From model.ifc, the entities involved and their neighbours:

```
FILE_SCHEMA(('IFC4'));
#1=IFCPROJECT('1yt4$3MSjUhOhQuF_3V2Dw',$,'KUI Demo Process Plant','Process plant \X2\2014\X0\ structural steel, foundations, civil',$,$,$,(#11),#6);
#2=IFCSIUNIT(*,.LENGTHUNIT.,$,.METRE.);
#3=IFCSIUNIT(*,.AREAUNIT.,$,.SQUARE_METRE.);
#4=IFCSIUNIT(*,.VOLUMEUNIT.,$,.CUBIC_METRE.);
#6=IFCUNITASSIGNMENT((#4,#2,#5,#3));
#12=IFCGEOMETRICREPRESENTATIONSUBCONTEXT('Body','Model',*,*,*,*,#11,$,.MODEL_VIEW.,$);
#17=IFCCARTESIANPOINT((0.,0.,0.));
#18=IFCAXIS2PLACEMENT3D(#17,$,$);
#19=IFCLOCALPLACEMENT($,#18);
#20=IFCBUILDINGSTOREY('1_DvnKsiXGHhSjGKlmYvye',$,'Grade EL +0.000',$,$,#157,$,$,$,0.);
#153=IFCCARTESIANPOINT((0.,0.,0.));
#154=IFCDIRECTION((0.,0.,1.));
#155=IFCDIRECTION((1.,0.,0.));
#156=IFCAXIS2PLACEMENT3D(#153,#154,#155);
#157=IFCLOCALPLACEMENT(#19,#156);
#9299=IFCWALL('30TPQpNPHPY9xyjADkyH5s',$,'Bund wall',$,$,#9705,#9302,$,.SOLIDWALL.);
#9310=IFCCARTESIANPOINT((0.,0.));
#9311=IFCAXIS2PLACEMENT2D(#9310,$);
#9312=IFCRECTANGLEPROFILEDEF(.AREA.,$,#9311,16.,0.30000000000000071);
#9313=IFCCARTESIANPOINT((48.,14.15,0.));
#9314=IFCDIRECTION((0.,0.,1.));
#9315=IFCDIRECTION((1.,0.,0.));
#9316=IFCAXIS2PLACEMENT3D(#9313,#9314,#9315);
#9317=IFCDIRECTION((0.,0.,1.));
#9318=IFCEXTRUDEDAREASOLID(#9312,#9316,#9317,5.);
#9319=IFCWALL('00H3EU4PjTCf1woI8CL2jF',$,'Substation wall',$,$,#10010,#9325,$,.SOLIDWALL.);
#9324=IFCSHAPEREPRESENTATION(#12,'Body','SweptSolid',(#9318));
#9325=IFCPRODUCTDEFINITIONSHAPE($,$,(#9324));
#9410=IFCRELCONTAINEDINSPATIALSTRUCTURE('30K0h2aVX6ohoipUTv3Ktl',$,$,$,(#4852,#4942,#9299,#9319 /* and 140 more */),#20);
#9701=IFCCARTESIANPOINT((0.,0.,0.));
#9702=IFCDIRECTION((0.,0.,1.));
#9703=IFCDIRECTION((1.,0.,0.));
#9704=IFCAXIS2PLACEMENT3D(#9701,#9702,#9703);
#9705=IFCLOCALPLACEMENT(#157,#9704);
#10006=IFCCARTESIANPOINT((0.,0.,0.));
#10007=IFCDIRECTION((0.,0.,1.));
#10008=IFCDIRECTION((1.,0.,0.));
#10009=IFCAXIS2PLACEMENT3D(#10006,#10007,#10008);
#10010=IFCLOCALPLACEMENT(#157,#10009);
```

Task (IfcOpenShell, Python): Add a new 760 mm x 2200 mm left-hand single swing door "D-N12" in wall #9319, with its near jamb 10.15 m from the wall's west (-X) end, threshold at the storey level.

```python
import numpy as np
import ifcopenshell
import ifcopenshell.api.feature
import ifcopenshell.api.geometry
import ifcopenshell.api.root
import ifcopenshell.api.spatial
import ifcopenshell.geom
import ifcopenshell.util.element
import ifcopenshell.util.placement
import ifcopenshell.util.representation
import ifcopenshell.util.shape
import ifcopenshell.util.unit

model = ifcopenshell.open("model.ifc")
unit_scale = ifcopenshell.util.unit.calculate_unit_scale(model)
settings = ifcopenshell.geom.settings()


def volume(element):
    """Net volume in cubic metres, openings subtracted."""
    shape = ifcopenshell.geom.create_shape(settings, element)
    return ifcopenshell.util.shape.get_volume(shape.geometry)


wall = model.by_id(9319)
storey = ifcopenshell.util.element.get_container(wall, ifc_class="IfcBuildingStorey")
context = ifcopenshell.util.representation.get_context(model, "Model", "Body", "MODEL_VIEW")
before = volume(wall)

width, height, from_end, sill = 0.76, 2.2, 10.15, 0.0  # metres

# The wall runs along its own X axis, and the end named is its -X end.
wall_shape = ifcopenshell.geom.create_shape(settings, wall)
x, y, z = ifcopenshell.util.shape.get_vertices(wall_shape.geometry).T
start = x.min() + from_end
face, thickness = float(y.min()), float(y.max() - y.min())
wall_matrix = ifcopenshell.util.placement.get_local_placement(wall.ObjectPlacement)
level = ifcopenshell.util.placement.get_local_placement(storey.ObjectPlacement)[2, 3]


def in_wall(x, y):
    """Placement at x, y metres in the wall's axes, at sill height."""
    matrix = wall_matrix.copy()
    matrix[:, 3] = wall_matrix @ np.array([x / unit_scale, y / unit_scale, 0.0, 1.0])
    matrix[2, 3] = level + sill / unit_scale
    return matrix


# Opening: a box that overshoots both wall faces by 50 mm.
opening = ifcopenshell.api.root.create_entity(model, ifc_class="IfcOpeningElement", predefined_type="OPENING")
box = ifcopenshell.api.geometry.add_wall_representation(
    model, context=context, length=width, height=height, thickness=thickness + 0.1
)
ifcopenshell.api.geometry.assign_representation(model, product=opening, representation=box)
ifcopenshell.api.geometry.edit_object_placement(model, product=opening, matrix=in_wall(start, face - 0.05), is_si=False)
ifcopenshell.api.feature.add_feature(model, feature=opening, element=wall)

door = ifcopenshell.api.root.create_entity(model, ifc_class="IfcDoor", name="D-N12", predefined_type="DOOR")
door.OverallWidth, door.OverallHeight = width / unit_scale, height / unit_scale
door.OperationType = "SINGLE_SWING_LEFT"
body = ifcopenshell.api.geometry.add_door_representation(
    model,
    context=context,
    overall_width=door.OverallWidth,
    overall_height=door.OverallHeight,
    operation_type="SINGLE_SWING_LEFT",
    lining_properties={"LiningDepth": thickness / unit_scale, "ThresholdDepth": thickness / unit_scale},
)
ifcopenshell.api.geometry.assign_representation(model, product=door, representation=body)
ifcopenshell.api.spatial.assign_container(model, products=[door], relating_structure=storey)
ifcopenshell.api.feature.add_filling(model, opening=opening, element=door)

# The lining spans the wall, so the door starts at the wall face.
ifcopenshell.api.geometry.edit_object_placement(model, product=door, matrix=in_wall(start, face), is_si=False)

after = volume(wall)

print(f"wall volume {before:.3f} -> {after:.3f} m3")

model.write("model_v2.ifc")
```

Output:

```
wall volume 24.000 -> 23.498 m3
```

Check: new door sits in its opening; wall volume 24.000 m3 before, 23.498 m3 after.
